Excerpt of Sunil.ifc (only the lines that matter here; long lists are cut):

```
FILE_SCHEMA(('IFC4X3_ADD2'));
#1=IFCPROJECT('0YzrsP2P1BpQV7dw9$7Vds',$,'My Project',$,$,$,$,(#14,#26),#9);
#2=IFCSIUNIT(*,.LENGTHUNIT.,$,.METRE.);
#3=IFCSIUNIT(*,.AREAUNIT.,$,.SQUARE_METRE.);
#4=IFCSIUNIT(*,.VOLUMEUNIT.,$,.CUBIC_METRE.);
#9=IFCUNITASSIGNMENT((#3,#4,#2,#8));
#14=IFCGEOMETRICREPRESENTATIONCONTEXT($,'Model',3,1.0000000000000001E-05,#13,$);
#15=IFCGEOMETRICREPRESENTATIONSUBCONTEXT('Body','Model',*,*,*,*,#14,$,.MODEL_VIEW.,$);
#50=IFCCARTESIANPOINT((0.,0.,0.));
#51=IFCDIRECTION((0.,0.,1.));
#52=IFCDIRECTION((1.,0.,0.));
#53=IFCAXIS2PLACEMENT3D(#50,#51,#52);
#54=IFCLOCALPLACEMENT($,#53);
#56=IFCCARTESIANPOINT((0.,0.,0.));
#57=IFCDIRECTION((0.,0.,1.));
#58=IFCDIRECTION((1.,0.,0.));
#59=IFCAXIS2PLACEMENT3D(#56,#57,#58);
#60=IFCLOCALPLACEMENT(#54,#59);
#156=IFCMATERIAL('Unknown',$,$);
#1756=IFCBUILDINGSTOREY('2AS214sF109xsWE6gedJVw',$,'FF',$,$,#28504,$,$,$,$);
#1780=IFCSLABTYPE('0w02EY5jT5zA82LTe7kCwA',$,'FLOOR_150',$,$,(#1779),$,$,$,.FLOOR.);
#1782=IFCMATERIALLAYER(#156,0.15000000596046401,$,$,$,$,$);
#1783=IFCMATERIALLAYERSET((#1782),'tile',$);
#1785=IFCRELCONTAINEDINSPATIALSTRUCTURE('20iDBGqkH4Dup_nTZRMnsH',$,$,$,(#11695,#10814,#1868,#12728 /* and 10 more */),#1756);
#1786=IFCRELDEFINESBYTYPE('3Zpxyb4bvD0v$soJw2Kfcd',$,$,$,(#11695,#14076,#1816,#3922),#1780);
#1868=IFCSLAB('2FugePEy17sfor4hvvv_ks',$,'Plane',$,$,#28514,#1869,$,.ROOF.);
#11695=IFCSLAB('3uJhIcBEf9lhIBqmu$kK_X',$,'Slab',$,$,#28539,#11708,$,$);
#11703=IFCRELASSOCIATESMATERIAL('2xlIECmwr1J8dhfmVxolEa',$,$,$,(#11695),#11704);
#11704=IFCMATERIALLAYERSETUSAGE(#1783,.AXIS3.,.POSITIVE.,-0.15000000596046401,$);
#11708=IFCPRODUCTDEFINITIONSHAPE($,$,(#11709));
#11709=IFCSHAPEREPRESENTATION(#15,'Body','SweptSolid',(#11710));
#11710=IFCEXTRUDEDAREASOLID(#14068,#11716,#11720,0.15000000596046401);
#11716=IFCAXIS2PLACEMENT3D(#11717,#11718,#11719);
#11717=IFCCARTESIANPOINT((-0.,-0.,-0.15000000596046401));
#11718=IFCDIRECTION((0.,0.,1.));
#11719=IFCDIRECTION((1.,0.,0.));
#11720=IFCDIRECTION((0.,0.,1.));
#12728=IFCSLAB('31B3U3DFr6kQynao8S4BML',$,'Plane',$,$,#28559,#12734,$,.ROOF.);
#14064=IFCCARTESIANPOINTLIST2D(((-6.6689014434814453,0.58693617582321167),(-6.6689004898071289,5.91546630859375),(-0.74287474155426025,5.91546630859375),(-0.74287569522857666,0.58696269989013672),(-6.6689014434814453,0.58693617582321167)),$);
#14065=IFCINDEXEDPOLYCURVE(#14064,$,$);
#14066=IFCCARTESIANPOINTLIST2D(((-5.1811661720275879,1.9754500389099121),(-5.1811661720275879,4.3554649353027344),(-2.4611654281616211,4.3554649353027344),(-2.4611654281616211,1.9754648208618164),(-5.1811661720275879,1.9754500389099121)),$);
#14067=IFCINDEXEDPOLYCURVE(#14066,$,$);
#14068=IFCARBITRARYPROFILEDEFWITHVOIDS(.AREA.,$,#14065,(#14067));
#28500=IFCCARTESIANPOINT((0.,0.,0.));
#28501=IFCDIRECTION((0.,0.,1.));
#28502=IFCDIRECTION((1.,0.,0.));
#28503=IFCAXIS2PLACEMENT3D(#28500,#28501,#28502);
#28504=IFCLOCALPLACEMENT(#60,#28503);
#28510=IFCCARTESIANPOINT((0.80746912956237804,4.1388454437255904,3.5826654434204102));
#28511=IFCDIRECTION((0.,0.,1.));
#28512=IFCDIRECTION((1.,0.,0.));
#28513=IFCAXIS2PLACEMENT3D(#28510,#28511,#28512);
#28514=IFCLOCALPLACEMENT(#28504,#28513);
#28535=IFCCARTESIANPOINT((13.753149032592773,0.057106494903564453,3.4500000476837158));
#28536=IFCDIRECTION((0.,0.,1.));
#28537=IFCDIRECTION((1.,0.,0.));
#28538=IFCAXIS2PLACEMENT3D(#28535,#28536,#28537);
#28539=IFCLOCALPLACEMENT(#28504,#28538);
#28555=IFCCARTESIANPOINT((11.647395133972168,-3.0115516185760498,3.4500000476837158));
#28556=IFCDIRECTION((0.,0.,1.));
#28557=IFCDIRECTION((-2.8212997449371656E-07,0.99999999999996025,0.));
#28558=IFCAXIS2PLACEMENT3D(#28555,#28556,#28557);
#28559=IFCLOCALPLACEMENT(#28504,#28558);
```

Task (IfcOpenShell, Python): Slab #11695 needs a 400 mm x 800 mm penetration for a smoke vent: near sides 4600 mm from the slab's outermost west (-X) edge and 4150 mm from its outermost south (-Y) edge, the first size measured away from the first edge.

```python
import numpy as np
import ifcopenshell
import ifcopenshell.api.feature
import ifcopenshell.api.geometry
import ifcopenshell.api.root
import ifcopenshell.geom
import ifcopenshell.util.placement
import ifcopenshell.util.representation
import ifcopenshell.util.shape
import ifcopenshell.util.unit

model = ifcopenshell.open("Sunil.ifc")
unit_scale = ifcopenshell.util.unit.calculate_unit_scale(model)
settings = ifcopenshell.geom.settings()


def volume(element):
    """Net volume in cubic metres, openings subtracted."""
    shape = ifcopenshell.geom.create_shape(settings, element)
    return ifcopenshell.util.shape.get_volume(shape.geometry)


slab = model.by_guid("3uJhIcBEf9lhIBqmu$kK_X")
before = volume(slab)

# Extent in the slab's own axes, in metres. The edges named are its -X and -Y sides.
slab_shape = ifcopenshell.geom.create_shape(settings, slab)
vertices = ifcopenshell.util.shape.get_vertices(slab_shape.geometry)
x_min, y_min, bottom = vertices.min(axis=0)
top = vertices[:, 2].max()

opening = ifcopenshell.api.root.create_entity(model, ifc_class="IfcOpeningElement", name="Smoke vent opening", predefined_type="OPENING")
context = ifcopenshell.util.representation.get_context(model, "Model", "Body", "MODEL_VIEW")
width, depth = 0.4, 0.8
outline = [(0.0, 0.0), (width, 0.0), (width, depth), (0.0, depth), (0.0, 0.0)]
# Overshoot both faces by 50 mm so the cut is clean.
shape = ifcopenshell.api.geometry.add_slab_representation(
    model, context=context, depth=top - bottom + 0.1, polyline=outline
)
ifcopenshell.api.geometry.assign_representation(model, product=opening, representation=shape)

matrix = ifcopenshell.util.placement.get_local_placement(slab.ObjectPlacement)
matrix[:, 3] = matrix @ np.append(np.array([x_min + 4.6, y_min + 4.15, bottom - 0.05]) / unit_scale, 1.0)
ifcopenshell.api.geometry.edit_object_placement(model, product=opening, matrix=matrix, is_si=False)
ifcopenshell.api.feature.add_feature(model, feature=opening, element=slab)

after = volume(slab)

print(f"slab volume {before:.3f} -> {after:.3f} m3")

model.write("Sunil-out.ifc")
```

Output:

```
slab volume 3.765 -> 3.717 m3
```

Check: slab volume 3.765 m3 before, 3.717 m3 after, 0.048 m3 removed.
